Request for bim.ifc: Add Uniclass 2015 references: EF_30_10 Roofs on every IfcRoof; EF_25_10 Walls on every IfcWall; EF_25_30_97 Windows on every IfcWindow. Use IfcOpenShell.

First a look at what the model holds.

```python
import ifcopenshell

model = ifcopenshell.open("bim.ifc")
print(model.schema)
print("classifications:", [c.Name for c in model.by_type("IfcClassification")])
for ifc_class in ("IfcDoor", "IfcRoof", "IfcStair", "IfcWall", "IfcWindow"):
    print(ifc_class, len(model.by_type(ifc_class)))
```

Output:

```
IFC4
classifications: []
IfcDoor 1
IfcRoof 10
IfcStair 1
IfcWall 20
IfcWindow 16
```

```python
import ifcopenshell
import ifcopenshell.api.classification

model = ifcopenshell.open("bim.ifc")

system = ifcopenshell.api.classification.add_classification(model, classification="Uniclass 2015")

codes = {
    "IfcRoof": ("EF_30_10", "Roofs"),
    "IfcWall": ("EF_25_10", "Walls"),
    "IfcWindow": ("EF_25_30_97", "Windows"),
}
for ifc_class, (code, name) in codes.items():
    products = model.by_type(ifc_class)
    ifcopenshell.api.classification.add_reference(
        model, products=products, classification=system, identification=code, name=name
    )
    print(code, len(products))

model.write("bim-out.ifc")
```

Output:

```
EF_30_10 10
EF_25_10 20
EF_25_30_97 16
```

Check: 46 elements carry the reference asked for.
